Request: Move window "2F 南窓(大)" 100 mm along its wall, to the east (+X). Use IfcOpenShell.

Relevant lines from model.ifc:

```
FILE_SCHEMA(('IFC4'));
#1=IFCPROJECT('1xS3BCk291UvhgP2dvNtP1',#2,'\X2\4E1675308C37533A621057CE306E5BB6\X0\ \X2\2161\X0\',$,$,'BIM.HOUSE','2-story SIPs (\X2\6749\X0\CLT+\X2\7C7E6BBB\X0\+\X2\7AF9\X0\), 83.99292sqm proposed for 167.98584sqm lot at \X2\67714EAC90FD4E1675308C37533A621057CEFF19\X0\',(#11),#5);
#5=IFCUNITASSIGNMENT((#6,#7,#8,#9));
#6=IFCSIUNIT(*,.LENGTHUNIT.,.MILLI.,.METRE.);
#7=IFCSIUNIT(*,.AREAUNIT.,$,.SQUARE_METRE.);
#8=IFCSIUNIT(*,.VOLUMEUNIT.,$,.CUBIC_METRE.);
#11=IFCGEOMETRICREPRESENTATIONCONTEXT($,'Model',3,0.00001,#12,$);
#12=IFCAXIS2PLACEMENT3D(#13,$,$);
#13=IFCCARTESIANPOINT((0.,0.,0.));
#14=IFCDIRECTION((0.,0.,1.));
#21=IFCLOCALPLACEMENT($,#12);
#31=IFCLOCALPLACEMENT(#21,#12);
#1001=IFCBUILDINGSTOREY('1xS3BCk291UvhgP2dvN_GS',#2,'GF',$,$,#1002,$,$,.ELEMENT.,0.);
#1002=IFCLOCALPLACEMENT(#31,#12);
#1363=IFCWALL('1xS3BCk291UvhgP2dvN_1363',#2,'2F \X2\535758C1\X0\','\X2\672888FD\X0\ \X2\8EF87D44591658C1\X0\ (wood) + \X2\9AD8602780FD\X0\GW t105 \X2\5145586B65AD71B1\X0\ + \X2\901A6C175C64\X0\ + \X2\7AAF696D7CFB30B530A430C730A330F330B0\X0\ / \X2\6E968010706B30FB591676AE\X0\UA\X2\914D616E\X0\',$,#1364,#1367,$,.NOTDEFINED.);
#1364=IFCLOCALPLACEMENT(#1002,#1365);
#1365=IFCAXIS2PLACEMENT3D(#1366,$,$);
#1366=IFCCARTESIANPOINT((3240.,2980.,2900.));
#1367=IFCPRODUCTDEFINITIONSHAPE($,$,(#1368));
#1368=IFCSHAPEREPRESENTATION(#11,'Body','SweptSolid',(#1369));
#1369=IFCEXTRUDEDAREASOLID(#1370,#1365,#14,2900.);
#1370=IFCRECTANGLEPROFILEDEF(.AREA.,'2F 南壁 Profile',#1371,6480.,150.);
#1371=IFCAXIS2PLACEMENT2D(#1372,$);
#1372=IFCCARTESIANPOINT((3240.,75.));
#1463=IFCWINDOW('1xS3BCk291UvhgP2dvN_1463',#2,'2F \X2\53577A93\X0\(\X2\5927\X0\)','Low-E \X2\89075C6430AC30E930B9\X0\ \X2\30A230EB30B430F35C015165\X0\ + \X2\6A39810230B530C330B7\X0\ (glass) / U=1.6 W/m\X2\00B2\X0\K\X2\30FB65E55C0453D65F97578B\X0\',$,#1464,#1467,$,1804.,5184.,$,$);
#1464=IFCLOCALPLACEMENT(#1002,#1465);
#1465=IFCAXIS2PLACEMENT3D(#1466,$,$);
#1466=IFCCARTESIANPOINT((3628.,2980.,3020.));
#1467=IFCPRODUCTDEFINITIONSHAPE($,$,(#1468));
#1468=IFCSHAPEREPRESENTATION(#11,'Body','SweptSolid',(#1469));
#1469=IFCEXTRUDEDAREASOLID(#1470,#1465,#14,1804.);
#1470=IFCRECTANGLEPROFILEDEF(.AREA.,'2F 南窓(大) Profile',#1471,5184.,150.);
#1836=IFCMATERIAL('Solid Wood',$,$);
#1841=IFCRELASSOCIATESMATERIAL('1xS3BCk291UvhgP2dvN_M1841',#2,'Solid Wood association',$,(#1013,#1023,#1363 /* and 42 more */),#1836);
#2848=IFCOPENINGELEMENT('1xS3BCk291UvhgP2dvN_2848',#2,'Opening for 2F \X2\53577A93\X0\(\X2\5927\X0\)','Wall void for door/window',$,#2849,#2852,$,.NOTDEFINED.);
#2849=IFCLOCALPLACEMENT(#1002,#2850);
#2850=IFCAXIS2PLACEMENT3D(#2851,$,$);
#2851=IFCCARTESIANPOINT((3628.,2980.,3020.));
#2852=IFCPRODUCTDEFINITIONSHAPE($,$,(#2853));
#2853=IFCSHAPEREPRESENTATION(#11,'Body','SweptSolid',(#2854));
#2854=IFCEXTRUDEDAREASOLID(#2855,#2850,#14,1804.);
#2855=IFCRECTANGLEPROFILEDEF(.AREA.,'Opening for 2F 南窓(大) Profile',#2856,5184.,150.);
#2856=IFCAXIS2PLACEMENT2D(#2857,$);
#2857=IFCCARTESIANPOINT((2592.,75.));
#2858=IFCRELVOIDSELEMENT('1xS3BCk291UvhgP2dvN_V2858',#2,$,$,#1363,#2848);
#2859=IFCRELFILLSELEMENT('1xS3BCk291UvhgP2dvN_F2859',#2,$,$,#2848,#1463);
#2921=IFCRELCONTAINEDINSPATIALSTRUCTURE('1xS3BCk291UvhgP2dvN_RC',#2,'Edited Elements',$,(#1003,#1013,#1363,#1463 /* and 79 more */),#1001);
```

```python
import ifcopenshell
import ifcopenshell.api.geometry
import ifcopenshell.util.placement
import ifcopenshell.util.unit

model = ifcopenshell.open("model.ifc")
unit_scale = ifcopenshell.util.unit.calculate_unit_scale(model)

window = model.by_guid("1xS3BCk291UvhgP2dvN_1463")
opening = window.FillsVoids[0].RelatingOpeningElement
wall = opening.VoidsElements[0].RelatingBuildingElement

wall_matrix = ifcopenshell.util.placement.get_local_placement(wall.ObjectPlacement)
shift = wall_matrix[:3, 0] * 0.1 / unit_scale
before = ifcopenshell.util.placement.get_local_placement(window.ObjectPlacement)[:3, 3].copy()

# The window is not placed relative to its opening, so move both.
for product in (opening, window):
    matrix = ifcopenshell.util.placement.get_local_placement(product.ObjectPlacement)
    matrix[:3, 3] += shift
    ifcopenshell.api.geometry.edit_object_placement(model, product=product, matrix=matrix, is_si=False)

after = ifcopenshell.util.placement.get_local_placement(window.ObjectPlacement)[:3, 3]
print("window moved by", (after - before).round(3) + 0.0)

model.write("model-out.ifc")
```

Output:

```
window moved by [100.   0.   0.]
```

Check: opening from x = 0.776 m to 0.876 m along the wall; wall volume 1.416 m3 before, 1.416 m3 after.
